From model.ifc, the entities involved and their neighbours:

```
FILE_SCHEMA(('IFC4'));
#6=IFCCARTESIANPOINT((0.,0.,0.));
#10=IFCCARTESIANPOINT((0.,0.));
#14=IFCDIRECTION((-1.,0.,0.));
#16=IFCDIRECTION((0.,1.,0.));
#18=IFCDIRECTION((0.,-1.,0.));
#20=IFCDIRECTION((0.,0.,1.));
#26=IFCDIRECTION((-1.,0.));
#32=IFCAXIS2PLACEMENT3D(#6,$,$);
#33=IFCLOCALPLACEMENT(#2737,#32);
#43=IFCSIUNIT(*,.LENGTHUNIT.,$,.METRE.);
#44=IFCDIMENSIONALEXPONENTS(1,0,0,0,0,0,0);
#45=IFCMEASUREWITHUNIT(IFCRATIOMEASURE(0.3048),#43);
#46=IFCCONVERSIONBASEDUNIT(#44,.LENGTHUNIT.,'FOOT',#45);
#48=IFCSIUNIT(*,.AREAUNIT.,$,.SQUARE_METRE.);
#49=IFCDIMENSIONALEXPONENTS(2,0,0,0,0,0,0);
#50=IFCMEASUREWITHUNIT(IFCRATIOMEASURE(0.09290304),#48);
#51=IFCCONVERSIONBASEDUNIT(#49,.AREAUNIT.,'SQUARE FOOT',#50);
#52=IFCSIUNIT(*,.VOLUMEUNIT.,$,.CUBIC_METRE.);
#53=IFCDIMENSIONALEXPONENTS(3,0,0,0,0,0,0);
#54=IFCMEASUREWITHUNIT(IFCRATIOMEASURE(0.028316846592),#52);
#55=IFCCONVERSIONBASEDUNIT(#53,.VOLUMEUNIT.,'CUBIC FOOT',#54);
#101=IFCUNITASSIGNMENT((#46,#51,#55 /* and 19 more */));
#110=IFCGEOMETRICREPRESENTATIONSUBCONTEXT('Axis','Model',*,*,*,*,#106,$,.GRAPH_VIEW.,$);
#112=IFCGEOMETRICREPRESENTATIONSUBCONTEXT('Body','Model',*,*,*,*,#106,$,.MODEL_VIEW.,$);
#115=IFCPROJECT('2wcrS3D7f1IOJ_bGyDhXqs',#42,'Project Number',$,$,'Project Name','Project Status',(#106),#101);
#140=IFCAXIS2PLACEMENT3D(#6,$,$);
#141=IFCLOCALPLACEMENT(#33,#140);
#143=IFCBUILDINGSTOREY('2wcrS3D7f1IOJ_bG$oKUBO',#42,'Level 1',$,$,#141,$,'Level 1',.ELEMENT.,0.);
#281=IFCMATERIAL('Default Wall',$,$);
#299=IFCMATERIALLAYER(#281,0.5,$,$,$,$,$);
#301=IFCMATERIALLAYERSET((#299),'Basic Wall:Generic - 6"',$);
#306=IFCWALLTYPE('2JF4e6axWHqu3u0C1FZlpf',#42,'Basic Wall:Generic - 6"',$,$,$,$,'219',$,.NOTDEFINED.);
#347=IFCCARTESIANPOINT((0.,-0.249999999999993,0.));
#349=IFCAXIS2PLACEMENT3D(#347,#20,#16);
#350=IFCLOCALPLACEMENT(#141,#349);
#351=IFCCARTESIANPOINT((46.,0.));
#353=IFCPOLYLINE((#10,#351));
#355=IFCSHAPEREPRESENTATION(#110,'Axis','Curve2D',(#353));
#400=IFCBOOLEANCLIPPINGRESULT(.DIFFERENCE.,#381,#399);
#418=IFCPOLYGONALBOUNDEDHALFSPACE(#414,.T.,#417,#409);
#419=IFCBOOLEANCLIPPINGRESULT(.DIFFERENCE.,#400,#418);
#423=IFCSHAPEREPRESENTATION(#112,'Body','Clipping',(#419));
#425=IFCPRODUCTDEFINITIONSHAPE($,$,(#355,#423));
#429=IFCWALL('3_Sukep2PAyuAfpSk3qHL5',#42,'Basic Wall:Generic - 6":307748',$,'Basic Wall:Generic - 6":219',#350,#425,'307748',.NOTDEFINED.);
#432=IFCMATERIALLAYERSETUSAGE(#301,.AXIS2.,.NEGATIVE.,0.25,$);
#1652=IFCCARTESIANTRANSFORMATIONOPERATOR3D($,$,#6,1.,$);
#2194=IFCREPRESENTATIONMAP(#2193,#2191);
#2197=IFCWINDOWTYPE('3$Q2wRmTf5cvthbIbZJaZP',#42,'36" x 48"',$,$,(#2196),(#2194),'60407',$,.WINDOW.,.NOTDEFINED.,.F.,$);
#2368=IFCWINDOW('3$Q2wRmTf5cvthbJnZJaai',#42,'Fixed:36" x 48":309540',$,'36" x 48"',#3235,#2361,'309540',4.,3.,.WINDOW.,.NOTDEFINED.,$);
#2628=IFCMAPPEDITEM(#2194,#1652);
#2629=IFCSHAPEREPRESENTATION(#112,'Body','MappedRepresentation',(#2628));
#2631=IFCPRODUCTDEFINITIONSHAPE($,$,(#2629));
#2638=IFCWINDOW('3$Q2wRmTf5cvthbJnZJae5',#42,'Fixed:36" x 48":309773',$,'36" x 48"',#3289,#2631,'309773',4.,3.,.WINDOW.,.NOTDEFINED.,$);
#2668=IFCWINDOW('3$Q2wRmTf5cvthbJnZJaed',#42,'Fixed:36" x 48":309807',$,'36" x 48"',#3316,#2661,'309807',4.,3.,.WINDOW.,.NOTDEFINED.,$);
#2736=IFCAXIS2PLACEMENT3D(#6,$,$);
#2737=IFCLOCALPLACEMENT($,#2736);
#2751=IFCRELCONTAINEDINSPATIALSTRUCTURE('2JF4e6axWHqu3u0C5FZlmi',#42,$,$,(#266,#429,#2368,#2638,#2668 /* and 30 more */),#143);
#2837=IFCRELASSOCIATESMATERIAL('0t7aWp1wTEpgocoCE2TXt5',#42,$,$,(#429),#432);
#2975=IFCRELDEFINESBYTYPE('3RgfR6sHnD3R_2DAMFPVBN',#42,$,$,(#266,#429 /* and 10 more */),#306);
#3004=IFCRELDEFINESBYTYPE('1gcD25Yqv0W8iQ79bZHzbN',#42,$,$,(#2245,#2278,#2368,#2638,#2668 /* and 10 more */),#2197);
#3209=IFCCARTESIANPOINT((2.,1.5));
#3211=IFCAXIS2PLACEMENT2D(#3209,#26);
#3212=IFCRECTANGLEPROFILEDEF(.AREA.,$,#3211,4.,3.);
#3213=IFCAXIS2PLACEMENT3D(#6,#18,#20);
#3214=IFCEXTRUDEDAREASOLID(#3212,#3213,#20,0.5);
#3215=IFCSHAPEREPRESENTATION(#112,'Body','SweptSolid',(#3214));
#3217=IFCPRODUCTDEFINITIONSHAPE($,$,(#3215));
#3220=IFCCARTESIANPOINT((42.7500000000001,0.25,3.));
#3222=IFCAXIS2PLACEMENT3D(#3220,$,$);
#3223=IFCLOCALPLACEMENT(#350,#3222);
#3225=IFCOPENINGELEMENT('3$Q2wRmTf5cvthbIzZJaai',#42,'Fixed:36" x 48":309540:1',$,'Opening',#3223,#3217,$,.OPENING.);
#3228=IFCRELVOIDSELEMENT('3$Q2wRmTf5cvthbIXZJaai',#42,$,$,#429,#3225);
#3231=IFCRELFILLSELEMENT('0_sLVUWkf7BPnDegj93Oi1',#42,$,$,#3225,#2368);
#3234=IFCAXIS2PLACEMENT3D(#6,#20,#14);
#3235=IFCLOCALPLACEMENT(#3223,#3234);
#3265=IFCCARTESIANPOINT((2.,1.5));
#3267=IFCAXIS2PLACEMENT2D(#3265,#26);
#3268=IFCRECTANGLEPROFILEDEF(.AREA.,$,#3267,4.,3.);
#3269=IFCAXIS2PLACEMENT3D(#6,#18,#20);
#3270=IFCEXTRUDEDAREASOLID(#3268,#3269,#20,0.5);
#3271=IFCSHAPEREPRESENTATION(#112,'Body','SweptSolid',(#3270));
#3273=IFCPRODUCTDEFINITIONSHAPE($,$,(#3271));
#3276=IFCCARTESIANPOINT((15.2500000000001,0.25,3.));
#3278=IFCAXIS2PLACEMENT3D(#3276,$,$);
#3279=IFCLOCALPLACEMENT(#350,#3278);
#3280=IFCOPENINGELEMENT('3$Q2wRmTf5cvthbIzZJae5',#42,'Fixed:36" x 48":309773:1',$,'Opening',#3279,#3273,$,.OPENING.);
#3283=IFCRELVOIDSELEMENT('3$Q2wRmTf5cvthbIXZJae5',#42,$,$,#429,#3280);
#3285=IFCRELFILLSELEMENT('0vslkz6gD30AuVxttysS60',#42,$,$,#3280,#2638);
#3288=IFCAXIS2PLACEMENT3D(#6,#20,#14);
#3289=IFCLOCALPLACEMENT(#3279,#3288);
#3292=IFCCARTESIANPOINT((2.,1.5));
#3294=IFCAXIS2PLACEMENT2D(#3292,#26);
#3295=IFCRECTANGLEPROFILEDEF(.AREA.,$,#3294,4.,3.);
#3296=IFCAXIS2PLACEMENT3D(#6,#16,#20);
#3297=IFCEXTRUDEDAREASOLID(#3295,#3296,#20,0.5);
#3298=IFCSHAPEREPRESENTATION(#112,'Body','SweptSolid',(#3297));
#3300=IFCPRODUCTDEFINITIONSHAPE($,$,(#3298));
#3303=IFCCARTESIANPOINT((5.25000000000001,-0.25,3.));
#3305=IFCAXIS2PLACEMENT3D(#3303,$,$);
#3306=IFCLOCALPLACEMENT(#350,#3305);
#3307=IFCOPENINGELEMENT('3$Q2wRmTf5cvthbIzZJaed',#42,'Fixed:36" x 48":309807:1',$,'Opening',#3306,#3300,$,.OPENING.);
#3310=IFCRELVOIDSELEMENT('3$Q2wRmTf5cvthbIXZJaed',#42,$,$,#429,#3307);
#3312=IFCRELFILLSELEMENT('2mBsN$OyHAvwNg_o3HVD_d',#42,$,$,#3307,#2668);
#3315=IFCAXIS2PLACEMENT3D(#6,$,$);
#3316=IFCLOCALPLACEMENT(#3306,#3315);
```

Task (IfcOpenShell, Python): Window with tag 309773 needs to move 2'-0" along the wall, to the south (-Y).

```python
import ifcopenshell
import ifcopenshell.api.geometry
import ifcopenshell.util.placement
import ifcopenshell.util.unit

model = ifcopenshell.open("model.ifc")
unit_scale = ifcopenshell.util.unit.calculate_unit_scale(model)

window = model.by_id(2638)
opening = window.FillsVoids[0].RelatingOpeningElement
wall = opening.VoidsElements[0].RelatingBuildingElement

wall_matrix = ifcopenshell.util.placement.get_local_placement(wall.ObjectPlacement)
shift = wall_matrix[:3, 0] * -24 * 0.0254 / unit_scale
before = ifcopenshell.util.placement.get_local_placement(window.ObjectPlacement)[:3, 3].copy()

# The window is placed relative to its opening, so it follows when the opening moves.
matrix = ifcopenshell.util.placement.get_local_placement(opening.ObjectPlacement)
matrix[:3, 3] += shift
ifcopenshell.api.geometry.edit_object_placement(
    model, product=opening, matrix=matrix, is_si=False, should_transform_children=True
)

after = ifcopenshell.util.placement.get_local_placement(window.ObjectPlacement)[:3, 3]
print("window moved by", (after - before).round(3) + 0.0)

model.write("model_rev.ifc")
```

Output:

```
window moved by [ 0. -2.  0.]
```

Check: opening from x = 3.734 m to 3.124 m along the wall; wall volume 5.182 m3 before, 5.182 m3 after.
